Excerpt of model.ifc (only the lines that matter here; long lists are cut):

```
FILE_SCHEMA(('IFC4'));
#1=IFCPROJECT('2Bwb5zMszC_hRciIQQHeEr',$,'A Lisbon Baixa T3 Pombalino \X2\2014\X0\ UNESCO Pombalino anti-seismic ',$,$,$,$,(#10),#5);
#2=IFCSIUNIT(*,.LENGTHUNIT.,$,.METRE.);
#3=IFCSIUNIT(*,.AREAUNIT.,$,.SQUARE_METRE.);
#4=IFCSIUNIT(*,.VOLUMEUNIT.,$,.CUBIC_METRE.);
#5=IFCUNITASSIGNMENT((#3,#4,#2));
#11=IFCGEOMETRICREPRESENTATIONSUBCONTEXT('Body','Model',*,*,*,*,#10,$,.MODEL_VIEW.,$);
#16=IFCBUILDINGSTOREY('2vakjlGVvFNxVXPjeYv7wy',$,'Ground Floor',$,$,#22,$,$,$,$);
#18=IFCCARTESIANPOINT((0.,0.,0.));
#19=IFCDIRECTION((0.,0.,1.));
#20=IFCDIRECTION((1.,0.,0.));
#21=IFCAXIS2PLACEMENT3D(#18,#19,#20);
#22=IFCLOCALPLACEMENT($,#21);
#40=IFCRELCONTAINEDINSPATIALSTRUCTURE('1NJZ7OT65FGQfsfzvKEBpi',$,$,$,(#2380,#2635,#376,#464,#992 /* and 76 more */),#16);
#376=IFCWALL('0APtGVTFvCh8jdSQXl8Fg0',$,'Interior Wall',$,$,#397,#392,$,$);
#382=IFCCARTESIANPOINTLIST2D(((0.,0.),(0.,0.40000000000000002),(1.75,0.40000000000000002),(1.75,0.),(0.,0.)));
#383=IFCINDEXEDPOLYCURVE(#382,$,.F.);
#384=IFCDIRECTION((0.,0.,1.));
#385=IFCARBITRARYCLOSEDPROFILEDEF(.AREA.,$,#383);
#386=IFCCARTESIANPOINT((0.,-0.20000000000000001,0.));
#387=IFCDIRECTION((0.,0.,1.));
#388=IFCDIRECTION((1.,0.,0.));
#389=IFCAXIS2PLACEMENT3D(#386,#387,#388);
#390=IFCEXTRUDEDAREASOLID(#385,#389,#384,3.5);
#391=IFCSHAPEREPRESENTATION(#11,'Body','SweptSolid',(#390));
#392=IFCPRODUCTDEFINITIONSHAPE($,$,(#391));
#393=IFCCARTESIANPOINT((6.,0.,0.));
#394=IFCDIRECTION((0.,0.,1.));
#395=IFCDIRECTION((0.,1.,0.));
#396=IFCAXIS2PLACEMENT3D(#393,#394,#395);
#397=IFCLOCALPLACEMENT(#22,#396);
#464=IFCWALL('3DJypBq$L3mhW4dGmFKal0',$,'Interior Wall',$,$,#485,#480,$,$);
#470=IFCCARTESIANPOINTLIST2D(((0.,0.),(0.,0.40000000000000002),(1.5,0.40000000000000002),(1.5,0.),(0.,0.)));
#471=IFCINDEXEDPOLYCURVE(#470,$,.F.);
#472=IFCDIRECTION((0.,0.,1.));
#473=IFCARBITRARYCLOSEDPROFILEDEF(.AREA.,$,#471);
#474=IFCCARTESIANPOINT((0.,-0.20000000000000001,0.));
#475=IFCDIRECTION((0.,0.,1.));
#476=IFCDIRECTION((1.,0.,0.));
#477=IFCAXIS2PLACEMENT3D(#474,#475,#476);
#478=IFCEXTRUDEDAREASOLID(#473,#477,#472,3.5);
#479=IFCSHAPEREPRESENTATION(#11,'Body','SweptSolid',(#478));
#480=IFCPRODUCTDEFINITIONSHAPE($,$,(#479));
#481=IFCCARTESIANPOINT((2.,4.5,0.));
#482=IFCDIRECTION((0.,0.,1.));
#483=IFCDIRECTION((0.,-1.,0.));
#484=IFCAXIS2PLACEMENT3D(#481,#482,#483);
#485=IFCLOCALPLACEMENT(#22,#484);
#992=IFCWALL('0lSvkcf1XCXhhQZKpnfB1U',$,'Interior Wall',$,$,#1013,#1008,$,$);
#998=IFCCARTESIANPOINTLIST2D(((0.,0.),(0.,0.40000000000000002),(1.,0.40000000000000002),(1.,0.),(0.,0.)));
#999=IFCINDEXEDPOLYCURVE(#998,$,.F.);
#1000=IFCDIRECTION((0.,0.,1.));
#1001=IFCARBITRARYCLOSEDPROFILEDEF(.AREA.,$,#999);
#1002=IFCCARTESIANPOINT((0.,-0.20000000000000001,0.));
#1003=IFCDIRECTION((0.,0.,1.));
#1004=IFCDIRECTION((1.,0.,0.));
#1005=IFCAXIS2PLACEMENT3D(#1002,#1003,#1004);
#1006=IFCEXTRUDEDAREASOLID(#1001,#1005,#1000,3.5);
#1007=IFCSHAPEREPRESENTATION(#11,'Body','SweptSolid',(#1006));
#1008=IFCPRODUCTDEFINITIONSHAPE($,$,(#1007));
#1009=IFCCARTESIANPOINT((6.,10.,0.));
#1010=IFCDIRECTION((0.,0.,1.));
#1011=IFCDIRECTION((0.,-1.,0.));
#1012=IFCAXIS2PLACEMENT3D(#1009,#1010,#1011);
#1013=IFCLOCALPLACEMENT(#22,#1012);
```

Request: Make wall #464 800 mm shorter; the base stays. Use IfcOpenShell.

```python
import ifcopenshell
import ifcopenshell.geom
import ifcopenshell.util.representation
import ifcopenshell.util.shape
import ifcopenshell.util.unit

model = ifcopenshell.open("model.ifc")
unit_scale = ifcopenshell.util.unit.calculate_unit_scale(model)
settings = ifcopenshell.geom.settings()


def volume(element):
    """Net volume in cubic metres, openings subtracted."""
    shape = ifcopenshell.geom.create_shape(settings, element)
    return ifcopenshell.util.shape.get_volume(shape.geometry)


wall = model.by_id(464)
before = volume(wall)

body = ifcopenshell.util.representation.get_representation(wall, "Model", "Body")
solid = body.Items[0]
old_height = solid.Depth
solid.Depth -= 0.8 / unit_scale
after = volume(wall)

print(f"height {old_height:g} -> {solid.Depth:g}, volume {before:.3f} -> {after:.3f} m3")

model.write("model_updated.ifc")
```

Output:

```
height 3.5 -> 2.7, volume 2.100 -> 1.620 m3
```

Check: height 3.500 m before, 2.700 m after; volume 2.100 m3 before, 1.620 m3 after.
